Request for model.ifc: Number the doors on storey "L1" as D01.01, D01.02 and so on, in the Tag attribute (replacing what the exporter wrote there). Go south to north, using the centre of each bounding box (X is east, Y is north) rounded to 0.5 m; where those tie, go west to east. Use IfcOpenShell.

First a look at what the model holds.

```python
import ifcopenshell
import ifcopenshell.util.element
import ifcopenshell.util.placement

model = ifcopenshell.open("model.ifc")
print(model.schema)
storey = next(s for s in model.by_type("IfcBuildingStorey") if s.Name == "L1")
doors = [e for e in ifcopenshell.util.element.get_decomposition(storey) if e.is_a("IfcDoor")]
for e in sorted(doors, key=lambda e: e.id()):
    origin = ifcopenshell.util.placement.get_local_placement(e.ObjectPlacement)[:3, 3]
    print(e.id(), e.Tag, e.Name, origin.round(2) + 0.0, sep=" | ")
```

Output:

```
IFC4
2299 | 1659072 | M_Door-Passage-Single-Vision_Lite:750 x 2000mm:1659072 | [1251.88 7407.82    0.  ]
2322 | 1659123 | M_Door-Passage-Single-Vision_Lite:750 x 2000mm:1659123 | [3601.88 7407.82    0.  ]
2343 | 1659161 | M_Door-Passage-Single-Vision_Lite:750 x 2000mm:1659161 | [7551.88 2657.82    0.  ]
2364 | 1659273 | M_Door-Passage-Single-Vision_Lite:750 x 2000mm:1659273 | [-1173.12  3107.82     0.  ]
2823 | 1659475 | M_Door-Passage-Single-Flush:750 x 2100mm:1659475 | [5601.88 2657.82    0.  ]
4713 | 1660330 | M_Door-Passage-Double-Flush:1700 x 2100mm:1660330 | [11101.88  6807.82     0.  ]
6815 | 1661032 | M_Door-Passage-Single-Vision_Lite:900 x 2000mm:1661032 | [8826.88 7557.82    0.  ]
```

```python
import ifcopenshell
import ifcopenshell.geom
import ifcopenshell.util.element
import ifcopenshell.util.shape

model = ifcopenshell.open("model.ifc")
settings = ifcopenshell.geom.settings()
settings.set("use-world-coords", True)


def centre(element):
    shape = ifcopenshell.geom.create_shape(settings, element)
    return ifcopenshell.util.shape.get_bbox_centroid(shape.geometry)


storey = next(s for s in model.by_type("IfcBuildingStorey") if s.Name == "L1")
doors = [e for e in ifcopenshell.util.element.get_decomposition(storey) if e.is_a("IfcDoor")]

# Insertion points can sit at a corner or the storey origin, so sort by the geometry (in metres).
centres = {e: centre(e) for e in doors}
doors.sort(key=lambda e: (round(centres[e][1] / 0.5), centres[e][0]))

for i, e in enumerate(doors, start=1):
    number = f"D01.{i:02d}"
    e.Tag = number
    print(e.id(), number)

model.write("model_rev.ifc")
```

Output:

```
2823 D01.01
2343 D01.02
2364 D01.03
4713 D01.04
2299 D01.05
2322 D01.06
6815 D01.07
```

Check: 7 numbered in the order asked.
